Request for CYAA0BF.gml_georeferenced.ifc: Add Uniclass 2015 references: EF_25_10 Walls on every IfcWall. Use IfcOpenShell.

First a look at what the model holds.

```python
import ifcopenshell

model = ifcopenshell.open("CYAA0BF.gml_georeferenced.ifc")
print(model.schema)
print("classifications:", [c.Name for c in model.by_type("IfcClassification")])
for ifc_class in ("IfcDoor", "IfcRoof", "IfcStair", "IfcWall", "IfcWindow"):
    print(ifc_class, len(model.by_type(ifc_class)))
```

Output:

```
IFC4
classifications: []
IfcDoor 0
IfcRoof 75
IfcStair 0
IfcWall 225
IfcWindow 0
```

```python
import ifcopenshell
import ifcopenshell.api.classification

model = ifcopenshell.open("CYAA0BF.gml_georeferenced.ifc")

system = ifcopenshell.api.classification.add_classification(model, classification="Uniclass 2015")

codes = {
    "IfcWall": ("EF_25_10", "Walls"),
}
for ifc_class, (code, name) in codes.items():
    products = model.by_type(ifc_class)
    ifcopenshell.api.classification.add_reference(
        model, products=products, classification=system, identification=code, name=name
    )
    print(code, len(products))

model.write("CYAA0BF.gml_georeferenced-out.ifc")
```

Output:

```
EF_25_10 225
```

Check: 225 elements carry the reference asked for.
